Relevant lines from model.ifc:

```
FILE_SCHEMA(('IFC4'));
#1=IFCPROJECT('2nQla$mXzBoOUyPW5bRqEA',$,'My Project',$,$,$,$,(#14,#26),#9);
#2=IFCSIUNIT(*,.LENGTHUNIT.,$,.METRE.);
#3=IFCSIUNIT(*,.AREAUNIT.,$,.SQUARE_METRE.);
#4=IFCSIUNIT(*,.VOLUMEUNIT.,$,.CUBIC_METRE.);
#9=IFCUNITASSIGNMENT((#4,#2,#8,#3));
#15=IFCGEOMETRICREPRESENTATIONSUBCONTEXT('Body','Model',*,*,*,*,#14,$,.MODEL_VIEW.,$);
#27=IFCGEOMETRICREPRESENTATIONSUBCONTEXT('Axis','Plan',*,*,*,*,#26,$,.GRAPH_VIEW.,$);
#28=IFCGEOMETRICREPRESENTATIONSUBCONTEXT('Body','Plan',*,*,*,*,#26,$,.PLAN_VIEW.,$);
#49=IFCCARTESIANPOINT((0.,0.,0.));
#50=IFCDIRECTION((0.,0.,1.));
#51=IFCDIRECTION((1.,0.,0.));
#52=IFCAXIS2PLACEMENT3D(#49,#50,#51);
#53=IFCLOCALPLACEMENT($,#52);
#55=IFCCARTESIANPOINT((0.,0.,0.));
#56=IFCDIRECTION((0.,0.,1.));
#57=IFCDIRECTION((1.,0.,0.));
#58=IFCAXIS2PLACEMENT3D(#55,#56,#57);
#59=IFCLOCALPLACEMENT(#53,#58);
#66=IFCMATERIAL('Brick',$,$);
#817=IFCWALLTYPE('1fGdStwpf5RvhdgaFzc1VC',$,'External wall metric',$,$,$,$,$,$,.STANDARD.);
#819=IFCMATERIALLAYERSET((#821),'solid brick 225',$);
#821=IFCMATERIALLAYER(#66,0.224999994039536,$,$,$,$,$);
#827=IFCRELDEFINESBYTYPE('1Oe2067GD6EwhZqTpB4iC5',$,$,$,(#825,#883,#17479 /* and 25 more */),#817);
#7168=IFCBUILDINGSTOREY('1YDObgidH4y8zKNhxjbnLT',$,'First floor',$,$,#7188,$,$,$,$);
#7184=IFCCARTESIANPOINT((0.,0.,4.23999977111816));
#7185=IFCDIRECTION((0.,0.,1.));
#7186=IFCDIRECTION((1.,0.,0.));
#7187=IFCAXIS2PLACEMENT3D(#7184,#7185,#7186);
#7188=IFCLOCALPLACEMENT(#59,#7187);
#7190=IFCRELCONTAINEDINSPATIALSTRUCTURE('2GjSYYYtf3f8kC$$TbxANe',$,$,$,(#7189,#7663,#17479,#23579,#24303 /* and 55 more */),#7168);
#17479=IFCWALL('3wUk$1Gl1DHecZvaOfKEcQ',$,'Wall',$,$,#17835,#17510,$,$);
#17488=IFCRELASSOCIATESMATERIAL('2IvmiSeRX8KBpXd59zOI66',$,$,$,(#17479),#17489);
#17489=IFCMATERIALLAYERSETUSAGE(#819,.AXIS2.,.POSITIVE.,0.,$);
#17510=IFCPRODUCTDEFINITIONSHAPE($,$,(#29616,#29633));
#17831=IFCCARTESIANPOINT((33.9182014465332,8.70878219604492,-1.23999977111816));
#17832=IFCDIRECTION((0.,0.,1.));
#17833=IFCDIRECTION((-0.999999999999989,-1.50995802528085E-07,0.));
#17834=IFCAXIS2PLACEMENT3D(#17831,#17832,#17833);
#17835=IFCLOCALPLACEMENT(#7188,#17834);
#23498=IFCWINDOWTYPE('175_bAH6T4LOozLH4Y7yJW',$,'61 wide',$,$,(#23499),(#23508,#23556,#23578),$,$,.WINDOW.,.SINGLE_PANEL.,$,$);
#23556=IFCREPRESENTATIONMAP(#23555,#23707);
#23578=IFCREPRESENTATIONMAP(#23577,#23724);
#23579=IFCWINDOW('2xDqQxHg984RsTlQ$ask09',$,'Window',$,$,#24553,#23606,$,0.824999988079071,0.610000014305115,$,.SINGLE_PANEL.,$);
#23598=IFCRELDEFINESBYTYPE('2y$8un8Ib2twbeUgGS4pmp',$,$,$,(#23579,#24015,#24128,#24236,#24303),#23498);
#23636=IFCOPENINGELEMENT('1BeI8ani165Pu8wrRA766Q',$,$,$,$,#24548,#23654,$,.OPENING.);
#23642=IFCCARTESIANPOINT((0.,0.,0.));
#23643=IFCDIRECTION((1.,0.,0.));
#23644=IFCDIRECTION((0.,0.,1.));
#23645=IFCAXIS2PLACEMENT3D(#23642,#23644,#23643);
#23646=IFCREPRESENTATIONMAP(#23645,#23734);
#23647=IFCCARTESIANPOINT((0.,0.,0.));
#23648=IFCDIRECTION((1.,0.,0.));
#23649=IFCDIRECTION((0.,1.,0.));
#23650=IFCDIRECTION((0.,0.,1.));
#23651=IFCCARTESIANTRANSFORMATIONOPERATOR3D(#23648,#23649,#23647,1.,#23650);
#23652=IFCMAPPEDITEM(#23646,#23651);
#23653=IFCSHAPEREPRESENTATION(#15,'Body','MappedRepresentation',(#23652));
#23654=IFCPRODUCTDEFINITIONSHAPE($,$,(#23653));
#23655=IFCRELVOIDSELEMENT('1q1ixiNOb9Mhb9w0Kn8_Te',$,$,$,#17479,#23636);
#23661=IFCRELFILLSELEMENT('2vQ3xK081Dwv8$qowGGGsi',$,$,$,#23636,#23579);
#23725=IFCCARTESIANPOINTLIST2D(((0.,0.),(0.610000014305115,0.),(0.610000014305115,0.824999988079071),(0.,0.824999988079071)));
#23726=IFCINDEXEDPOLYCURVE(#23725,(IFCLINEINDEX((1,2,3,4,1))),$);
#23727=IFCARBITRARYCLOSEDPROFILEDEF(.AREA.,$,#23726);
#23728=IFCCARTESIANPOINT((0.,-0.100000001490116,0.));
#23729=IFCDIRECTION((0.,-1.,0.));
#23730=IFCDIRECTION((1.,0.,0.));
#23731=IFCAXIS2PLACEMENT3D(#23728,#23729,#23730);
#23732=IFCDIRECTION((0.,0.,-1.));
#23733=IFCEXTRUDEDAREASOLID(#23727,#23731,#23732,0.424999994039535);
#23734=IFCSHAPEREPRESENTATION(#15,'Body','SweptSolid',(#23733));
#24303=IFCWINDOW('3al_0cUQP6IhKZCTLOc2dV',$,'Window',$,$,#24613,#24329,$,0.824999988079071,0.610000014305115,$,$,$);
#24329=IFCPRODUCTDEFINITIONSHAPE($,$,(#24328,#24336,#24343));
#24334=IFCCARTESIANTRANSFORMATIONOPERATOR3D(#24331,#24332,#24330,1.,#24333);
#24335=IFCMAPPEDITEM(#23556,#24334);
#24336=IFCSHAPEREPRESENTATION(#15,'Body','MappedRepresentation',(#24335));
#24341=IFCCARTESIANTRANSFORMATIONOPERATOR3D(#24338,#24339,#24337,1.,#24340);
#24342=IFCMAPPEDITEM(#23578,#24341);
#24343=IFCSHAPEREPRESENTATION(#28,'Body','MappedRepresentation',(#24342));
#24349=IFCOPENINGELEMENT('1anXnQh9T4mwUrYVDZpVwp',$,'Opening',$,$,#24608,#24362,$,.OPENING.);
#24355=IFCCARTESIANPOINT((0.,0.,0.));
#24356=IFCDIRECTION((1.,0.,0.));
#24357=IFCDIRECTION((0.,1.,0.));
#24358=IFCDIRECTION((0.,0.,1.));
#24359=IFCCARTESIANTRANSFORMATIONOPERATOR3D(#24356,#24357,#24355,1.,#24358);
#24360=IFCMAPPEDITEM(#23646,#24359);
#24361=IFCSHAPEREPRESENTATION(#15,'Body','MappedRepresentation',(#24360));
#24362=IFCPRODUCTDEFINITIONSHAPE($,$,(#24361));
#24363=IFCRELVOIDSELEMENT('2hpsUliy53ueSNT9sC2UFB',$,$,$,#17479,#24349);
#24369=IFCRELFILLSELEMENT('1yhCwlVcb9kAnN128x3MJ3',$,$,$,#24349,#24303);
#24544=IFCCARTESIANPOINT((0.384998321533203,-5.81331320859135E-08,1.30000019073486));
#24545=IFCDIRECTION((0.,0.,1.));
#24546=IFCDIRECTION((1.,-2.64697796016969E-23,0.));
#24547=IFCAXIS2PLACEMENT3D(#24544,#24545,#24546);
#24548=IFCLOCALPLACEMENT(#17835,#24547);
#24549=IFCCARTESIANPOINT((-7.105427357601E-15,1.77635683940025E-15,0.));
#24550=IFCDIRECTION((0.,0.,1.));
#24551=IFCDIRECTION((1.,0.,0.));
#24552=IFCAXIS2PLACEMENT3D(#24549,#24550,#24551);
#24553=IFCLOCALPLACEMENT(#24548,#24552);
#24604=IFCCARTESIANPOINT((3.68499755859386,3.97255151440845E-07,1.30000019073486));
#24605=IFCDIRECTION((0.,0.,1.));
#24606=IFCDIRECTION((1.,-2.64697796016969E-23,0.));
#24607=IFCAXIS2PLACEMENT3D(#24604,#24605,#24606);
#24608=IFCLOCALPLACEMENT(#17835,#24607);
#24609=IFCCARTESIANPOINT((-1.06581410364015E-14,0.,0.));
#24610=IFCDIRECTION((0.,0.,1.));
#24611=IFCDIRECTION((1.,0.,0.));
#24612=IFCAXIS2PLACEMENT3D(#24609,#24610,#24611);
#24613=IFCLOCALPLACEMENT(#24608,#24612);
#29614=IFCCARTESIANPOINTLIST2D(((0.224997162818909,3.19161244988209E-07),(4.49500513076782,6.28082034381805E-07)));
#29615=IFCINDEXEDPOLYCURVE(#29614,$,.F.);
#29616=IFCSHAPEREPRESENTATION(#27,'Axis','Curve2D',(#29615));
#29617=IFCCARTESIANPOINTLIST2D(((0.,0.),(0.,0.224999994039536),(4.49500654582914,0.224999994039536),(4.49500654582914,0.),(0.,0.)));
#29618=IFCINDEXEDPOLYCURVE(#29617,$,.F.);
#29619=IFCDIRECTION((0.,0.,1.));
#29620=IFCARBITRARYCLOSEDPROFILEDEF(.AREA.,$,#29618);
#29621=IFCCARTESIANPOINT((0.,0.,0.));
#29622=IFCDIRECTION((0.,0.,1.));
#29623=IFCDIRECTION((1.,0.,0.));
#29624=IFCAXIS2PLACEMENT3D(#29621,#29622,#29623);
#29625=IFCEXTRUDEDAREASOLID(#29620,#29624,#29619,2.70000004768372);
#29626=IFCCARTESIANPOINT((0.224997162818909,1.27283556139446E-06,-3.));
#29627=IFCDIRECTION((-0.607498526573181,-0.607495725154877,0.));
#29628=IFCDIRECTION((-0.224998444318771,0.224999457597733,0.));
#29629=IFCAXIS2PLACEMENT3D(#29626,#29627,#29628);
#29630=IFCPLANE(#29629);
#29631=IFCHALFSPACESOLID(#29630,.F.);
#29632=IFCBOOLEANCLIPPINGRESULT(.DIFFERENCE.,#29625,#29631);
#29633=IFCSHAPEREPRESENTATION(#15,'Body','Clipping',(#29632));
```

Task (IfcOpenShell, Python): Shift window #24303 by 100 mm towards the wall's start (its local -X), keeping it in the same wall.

```python
import ifcopenshell
import ifcopenshell.api.geometry
import ifcopenshell.util.placement
import ifcopenshell.util.unit

model = ifcopenshell.open("model.ifc")
unit_scale = ifcopenshell.util.unit.calculate_unit_scale(model)

window = model.by_guid("3al_0cUQP6IhKZCTLOc2dV")
opening = window.FillsVoids[0].RelatingOpeningElement
wall = opening.VoidsElements[0].RelatingBuildingElement

wall_matrix = ifcopenshell.util.placement.get_local_placement(wall.ObjectPlacement)
shift = wall_matrix[:3, 0] * -0.1 / unit_scale
before = ifcopenshell.util.placement.get_local_placement(window.ObjectPlacement)[:3, 3].copy()

# The window is placed relative to its opening, so it follows when the opening moves.
matrix = ifcopenshell.util.placement.get_local_placement(opening.ObjectPlacement)
matrix[:3, 3] += shift
ifcopenshell.api.geometry.edit_object_placement(
    model, product=opening, matrix=matrix, is_si=False, should_transform_children=True
)

after = ifcopenshell.util.placement.get_local_placement(window.ObjectPlacement)[:3, 3]
print("window moved by", (after - before).round(3) + 0.0)

model.write("model-out.ifc")
```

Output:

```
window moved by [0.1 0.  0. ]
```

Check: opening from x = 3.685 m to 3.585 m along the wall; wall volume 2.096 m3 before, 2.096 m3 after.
